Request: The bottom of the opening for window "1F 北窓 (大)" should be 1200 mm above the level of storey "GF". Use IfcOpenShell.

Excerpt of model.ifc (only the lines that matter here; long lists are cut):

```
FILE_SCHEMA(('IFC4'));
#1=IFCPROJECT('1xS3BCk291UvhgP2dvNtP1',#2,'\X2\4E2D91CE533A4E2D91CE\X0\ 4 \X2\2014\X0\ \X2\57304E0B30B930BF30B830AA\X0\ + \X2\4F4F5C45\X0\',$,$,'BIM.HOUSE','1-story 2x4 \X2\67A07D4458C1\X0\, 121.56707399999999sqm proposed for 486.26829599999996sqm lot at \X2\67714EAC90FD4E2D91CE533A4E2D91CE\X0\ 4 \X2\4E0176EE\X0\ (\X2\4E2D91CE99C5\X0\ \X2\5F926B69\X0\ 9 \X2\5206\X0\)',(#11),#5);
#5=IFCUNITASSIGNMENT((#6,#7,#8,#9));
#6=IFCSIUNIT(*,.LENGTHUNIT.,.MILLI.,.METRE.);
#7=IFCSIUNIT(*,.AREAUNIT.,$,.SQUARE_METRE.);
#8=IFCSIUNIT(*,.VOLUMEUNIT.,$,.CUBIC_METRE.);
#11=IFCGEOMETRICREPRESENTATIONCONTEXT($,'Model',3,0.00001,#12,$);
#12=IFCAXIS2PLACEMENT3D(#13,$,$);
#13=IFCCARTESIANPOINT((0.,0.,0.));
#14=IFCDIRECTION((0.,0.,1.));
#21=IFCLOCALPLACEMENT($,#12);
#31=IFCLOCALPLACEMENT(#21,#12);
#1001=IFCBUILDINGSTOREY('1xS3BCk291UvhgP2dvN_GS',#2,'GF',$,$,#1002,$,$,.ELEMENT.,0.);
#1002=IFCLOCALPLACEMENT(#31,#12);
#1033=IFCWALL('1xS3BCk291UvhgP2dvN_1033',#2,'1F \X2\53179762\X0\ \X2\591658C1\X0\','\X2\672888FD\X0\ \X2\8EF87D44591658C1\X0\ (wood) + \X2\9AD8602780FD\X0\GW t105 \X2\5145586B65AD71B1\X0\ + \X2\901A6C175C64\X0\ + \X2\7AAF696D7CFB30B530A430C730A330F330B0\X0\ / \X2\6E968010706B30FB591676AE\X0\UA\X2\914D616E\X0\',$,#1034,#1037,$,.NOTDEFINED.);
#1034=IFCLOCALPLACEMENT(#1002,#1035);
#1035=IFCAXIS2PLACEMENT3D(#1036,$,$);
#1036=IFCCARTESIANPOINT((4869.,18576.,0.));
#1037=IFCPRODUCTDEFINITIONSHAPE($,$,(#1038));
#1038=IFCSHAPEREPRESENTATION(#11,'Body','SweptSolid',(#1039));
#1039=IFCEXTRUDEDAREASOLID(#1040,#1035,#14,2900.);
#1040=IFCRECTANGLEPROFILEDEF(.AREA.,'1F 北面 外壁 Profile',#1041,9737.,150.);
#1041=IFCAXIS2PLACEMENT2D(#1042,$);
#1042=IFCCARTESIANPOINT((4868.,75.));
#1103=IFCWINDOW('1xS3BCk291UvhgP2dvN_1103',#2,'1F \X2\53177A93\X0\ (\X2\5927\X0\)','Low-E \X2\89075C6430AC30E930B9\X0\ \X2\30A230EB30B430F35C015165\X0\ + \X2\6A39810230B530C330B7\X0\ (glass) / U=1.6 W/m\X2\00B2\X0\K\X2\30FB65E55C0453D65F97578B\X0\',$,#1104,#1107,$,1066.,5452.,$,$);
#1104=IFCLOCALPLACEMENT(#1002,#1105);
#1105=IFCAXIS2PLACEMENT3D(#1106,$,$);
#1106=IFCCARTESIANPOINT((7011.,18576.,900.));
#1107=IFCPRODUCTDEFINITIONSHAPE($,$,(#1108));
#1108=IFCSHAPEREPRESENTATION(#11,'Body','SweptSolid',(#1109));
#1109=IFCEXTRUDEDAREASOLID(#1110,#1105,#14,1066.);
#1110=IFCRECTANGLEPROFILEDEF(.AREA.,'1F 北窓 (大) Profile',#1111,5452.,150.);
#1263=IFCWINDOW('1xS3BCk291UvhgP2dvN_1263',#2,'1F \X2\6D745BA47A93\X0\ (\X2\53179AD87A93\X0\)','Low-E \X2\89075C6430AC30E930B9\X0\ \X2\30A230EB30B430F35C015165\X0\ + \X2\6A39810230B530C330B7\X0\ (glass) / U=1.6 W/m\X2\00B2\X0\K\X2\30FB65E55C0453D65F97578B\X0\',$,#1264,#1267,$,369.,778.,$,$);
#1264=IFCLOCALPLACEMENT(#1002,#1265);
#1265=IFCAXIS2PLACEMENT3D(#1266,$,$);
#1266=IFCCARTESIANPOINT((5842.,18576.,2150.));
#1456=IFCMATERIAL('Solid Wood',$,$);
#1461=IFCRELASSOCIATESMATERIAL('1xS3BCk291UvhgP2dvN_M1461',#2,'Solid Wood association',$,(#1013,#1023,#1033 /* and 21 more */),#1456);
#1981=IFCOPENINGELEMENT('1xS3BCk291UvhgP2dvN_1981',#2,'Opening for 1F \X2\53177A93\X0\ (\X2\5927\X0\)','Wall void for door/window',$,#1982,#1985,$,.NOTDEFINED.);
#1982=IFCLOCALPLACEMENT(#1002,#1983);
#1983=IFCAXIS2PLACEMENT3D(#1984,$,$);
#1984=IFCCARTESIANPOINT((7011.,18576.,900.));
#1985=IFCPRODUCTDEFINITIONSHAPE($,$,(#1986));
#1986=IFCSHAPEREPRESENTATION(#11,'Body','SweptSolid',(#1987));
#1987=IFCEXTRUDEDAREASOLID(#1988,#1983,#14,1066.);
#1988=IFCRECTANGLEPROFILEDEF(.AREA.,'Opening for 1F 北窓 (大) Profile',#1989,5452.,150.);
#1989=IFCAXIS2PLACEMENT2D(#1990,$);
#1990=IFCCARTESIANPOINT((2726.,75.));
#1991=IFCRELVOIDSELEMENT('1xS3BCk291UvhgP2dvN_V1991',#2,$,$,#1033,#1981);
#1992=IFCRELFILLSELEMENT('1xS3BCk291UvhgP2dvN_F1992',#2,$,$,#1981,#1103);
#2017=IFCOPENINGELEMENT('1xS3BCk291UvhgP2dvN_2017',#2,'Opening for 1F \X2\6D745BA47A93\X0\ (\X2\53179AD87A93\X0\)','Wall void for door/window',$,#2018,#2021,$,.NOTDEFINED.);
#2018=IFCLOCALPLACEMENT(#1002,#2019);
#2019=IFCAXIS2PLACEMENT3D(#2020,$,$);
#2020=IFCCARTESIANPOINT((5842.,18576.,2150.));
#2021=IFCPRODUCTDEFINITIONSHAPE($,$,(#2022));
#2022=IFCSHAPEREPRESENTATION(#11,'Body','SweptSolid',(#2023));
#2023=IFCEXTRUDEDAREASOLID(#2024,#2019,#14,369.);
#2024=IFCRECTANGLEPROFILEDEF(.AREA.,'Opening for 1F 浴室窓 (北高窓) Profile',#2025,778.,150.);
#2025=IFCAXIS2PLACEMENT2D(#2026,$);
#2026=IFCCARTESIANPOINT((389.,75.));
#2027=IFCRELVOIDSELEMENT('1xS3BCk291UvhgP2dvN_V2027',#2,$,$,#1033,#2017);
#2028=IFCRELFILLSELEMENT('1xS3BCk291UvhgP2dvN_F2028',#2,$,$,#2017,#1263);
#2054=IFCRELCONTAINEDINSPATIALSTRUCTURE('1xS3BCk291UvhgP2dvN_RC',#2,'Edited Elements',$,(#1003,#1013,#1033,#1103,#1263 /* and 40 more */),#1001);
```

```python
import numpy as np
import ifcopenshell
import ifcopenshell.api.geometry
import ifcopenshell.geom
import ifcopenshell.util.element
import ifcopenshell.util.placement
import ifcopenshell.util.shape
import ifcopenshell.util.unit

model = ifcopenshell.open("model.ifc")
unit_scale = ifcopenshell.util.unit.calculate_unit_scale(model)

window = model.by_guid("1xS3BCk291UvhgP2dvN_1103")
opening = window.FillsVoids[0].RelatingOpeningElement
storey = ifcopenshell.util.element.get_container(window, ifc_class="IfcBuildingStorey")
level = ifcopenshell.util.placement.get_local_placement(storey.ObjectPlacement)[2, 3]

# The opening's origin need not be at the sill, so measure its lowest point.
shape = ifcopenshell.geom.create_shape(ifcopenshell.geom.settings(), opening)
bottom = ifcopenshell.util.shape.get_shape_bottom_elevation(shape, shape.geometry) / unit_scale
dz = level + 1200.0 - bottom

shift = np.array([0.0, 0.0, dz])
# The window is not placed relative to its opening, so move both.
for product in (opening, window):
    matrix = ifcopenshell.util.placement.get_local_placement(product.ObjectPlacement)
    matrix[:3, 3] += shift
    ifcopenshell.api.geometry.edit_object_placement(model, product=product, matrix=matrix, is_si=False)

print(f"moved by {dz * unit_scale:+.3f} m")

model.write("model-out.ifc")
```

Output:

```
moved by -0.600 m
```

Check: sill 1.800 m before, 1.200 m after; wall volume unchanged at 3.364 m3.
